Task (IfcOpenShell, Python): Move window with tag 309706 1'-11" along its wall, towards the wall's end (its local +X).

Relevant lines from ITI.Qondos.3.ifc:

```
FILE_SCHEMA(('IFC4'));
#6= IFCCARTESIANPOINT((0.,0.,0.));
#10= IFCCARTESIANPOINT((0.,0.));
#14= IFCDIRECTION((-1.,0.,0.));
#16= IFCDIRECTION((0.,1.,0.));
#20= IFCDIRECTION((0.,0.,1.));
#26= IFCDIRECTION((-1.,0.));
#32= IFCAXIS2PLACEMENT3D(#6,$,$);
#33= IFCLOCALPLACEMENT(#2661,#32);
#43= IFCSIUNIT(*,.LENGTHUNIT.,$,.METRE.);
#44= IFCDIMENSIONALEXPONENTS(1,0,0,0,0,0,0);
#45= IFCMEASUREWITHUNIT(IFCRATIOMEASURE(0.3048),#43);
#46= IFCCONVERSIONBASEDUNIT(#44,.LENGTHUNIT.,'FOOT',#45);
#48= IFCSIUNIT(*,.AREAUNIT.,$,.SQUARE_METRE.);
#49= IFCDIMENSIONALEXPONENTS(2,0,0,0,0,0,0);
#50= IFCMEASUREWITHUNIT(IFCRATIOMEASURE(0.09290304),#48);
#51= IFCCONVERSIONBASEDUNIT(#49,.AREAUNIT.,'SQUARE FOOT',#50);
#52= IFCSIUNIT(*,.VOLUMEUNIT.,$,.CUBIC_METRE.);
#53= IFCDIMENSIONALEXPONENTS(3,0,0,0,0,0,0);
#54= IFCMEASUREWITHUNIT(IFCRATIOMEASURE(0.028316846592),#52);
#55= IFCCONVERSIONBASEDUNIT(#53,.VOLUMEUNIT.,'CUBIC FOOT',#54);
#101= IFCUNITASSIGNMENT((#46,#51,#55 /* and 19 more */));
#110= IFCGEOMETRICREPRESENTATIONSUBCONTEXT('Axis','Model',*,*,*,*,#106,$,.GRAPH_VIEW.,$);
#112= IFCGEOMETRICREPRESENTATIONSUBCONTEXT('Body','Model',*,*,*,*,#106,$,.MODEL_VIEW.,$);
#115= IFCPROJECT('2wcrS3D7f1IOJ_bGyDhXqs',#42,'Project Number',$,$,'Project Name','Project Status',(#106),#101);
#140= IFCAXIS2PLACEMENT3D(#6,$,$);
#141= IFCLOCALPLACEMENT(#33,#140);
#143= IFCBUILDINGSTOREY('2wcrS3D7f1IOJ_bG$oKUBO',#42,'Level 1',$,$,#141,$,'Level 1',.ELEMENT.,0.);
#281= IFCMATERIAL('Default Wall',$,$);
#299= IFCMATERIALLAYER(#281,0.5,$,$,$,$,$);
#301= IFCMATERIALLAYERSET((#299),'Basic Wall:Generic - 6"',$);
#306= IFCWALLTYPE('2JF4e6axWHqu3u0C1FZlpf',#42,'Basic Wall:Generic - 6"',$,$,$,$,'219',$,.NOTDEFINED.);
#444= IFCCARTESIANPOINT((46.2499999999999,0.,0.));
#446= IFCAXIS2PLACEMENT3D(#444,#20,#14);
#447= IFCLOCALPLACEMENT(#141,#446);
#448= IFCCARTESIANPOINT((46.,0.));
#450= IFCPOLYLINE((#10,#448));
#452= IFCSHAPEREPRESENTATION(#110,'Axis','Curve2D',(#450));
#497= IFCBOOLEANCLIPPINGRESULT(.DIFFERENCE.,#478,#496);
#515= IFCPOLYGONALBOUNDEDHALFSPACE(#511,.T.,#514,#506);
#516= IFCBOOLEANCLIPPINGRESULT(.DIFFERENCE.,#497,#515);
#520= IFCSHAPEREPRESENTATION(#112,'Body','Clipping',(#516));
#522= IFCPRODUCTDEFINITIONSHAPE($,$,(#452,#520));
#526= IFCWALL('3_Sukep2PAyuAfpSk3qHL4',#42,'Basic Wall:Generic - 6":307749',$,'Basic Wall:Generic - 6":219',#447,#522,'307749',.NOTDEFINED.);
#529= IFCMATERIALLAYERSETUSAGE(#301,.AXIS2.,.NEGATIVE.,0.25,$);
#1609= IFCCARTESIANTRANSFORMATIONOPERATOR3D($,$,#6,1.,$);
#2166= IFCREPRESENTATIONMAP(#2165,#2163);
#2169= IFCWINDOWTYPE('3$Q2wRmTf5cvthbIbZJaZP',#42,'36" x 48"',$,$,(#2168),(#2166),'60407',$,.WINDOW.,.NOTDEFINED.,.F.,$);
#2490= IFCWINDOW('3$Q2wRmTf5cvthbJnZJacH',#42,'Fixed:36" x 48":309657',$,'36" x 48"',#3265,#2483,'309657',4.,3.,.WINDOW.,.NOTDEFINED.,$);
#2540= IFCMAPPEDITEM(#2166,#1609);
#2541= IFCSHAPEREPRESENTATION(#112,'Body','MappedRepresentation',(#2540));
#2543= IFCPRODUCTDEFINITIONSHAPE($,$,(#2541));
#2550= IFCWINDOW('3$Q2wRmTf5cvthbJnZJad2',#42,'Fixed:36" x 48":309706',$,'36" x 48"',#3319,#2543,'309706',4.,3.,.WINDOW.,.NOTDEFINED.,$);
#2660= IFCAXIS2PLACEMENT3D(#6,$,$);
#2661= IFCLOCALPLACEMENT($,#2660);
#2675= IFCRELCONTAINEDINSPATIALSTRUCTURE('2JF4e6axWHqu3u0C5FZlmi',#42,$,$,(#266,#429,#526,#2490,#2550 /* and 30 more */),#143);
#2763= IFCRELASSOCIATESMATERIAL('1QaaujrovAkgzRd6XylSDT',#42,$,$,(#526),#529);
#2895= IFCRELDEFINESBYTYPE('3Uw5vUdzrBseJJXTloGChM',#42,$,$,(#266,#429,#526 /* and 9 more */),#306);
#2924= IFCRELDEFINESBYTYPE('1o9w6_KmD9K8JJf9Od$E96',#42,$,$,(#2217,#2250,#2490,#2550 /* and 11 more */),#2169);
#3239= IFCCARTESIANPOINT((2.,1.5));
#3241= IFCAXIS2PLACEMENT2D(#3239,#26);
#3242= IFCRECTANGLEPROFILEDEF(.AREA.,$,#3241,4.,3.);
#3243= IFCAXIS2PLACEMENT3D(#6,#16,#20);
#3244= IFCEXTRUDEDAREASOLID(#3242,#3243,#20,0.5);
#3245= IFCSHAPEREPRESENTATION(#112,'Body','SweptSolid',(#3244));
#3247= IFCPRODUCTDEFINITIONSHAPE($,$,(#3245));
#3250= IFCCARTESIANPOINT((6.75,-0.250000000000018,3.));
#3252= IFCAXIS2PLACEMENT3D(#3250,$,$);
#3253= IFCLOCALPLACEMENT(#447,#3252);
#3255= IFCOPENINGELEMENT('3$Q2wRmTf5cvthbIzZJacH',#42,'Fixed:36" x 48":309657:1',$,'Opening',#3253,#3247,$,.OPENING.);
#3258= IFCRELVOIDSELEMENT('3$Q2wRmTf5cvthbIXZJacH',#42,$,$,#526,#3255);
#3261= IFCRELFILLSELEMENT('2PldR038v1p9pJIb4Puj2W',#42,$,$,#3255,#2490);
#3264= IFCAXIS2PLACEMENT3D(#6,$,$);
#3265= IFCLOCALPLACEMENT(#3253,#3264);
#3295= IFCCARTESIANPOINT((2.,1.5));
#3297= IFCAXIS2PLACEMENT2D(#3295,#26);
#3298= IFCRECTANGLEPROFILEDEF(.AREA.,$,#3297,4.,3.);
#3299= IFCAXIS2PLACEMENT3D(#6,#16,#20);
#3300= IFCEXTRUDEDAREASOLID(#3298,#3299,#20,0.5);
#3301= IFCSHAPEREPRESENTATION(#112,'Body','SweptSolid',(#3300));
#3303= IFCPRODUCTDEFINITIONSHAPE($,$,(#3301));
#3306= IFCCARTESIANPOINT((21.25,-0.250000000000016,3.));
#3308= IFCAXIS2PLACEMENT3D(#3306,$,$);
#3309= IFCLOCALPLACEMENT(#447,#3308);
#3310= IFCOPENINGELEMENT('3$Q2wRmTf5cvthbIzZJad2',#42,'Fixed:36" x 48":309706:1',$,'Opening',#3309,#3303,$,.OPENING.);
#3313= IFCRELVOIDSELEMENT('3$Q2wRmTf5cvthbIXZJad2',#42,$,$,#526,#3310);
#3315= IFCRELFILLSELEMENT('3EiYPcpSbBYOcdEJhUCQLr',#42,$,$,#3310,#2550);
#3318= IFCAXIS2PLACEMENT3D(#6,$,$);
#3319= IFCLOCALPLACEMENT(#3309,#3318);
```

```python
import ifcopenshell
import ifcopenshell.api.geometry
import ifcopenshell.util.placement
import ifcopenshell.util.unit

model = ifcopenshell.open("ITI.Qondos.3.ifc")
unit_scale = ifcopenshell.util.unit.calculate_unit_scale(model)

window = model.by_guid("3$Q2wRmTf5cvthbJnZJad2")
opening = window.FillsVoids[0].RelatingOpeningElement
wall = opening.VoidsElements[0].RelatingBuildingElement

wall_matrix = ifcopenshell.util.placement.get_local_placement(wall.ObjectPlacement)
shift = wall_matrix[:3, 0] * 23 * 0.0254 / unit_scale
before = ifcopenshell.util.placement.get_local_placement(window.ObjectPlacement)[:3, 3].copy()

# The window is placed relative to its opening, so it follows when the opening moves.
matrix = ifcopenshell.util.placement.get_local_placement(opening.ObjectPlacement)
matrix[:3, 3] += shift
ifcopenshell.api.geometry.edit_object_placement(
    model, product=opening, matrix=matrix, is_si=False, should_transform_children=True
)

after = ifcopenshell.util.placement.get_local_placement(window.ObjectPlacement)[:3, 3]
print("window moved by", (after - before).round(3) + 0.0)

model.write("ITI.Qondos.3_rev.ifc")
```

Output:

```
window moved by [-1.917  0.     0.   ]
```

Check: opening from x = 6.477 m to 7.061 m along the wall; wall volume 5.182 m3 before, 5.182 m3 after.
